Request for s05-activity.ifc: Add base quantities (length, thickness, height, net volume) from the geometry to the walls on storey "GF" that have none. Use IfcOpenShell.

First a look at what the model holds.

```python
import ifcopenshell
import ifcopenshell.util.element
import ifcopenshell.util.unit

model = ifcopenshell.open("s05-activity.ifc")
print(model.schema)
for unit_type in ("LENGTHUNIT", "AREAUNIT", "VOLUMEUNIT"):
    print(unit_type, ifcopenshell.util.unit.calculate_unit_scale(model, unit_type))
storey = next(s for s in model.by_type("IfcBuildingStorey") if s.Name == "GF")
walls = [e for e in ifcopenshell.util.element.get_decomposition(storey) if e.is_a("IfcWall")]
for e in sorted(walls, key=lambda e: e.id()):
    print(e.id(), e.is_a(), e.Name, list(ifcopenshell.util.element.get_psets(e, qtos_only=True)), sep=" | ")
```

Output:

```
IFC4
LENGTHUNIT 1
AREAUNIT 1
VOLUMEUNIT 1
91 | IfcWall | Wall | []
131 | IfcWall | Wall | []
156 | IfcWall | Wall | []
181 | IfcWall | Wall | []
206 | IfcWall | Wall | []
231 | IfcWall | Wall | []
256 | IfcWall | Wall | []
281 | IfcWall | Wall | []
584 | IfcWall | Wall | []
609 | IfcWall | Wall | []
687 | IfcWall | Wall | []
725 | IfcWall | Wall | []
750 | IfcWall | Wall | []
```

```python
import ifcopenshell
import ifcopenshell.api.pset
import ifcopenshell.geom
import ifcopenshell.util.element
import ifcopenshell.util.shape
import ifcopenshell.util.unit

model = ifcopenshell.open("s05-activity.ifc")
unit_scale = ifcopenshell.util.unit.calculate_unit_scale(model)
volume_scale = ifcopenshell.util.unit.calculate_unit_scale(model, "VOLUMEUNIT")
settings = ifcopenshell.geom.settings()

storey = next(s for s in model.by_type("IfcBuildingStorey") if s.Name == "GF")
walls = [e for e in ifcopenshell.util.element.get_decomposition(storey) if e.is_a("IfcWall")]

for e in sorted(walls, key=lambda e: e.id()):
    if ifcopenshell.util.element.get_psets(e, qtos_only=True, should_inherit=False):
        continue
    # Geometry comes back in metres, in the element's own axes.
    shape = ifcopenshell.geom.create_shape(settings, e)
    values = {
        "Length": ifcopenshell.util.shape.get_x(shape.geometry) / unit_scale,
        "Width": ifcopenshell.util.shape.get_y(shape.geometry) / unit_scale,
        "Height": ifcopenshell.util.shape.get_z(shape.geometry) / unit_scale,
        "NetVolume": ifcopenshell.util.shape.get_volume(shape.geometry) / volume_scale,
    }
    qto = ifcopenshell.api.pset.add_qto(model, product=e, name="Qto_WallBaseQuantities")
    ifcopenshell.api.pset.edit_qto(model, qto=qto, properties=values)
    print(e.id(), {k: round(v, 3) for k, v in values.items()})

model.write("s05-activity_updated.ifc")
```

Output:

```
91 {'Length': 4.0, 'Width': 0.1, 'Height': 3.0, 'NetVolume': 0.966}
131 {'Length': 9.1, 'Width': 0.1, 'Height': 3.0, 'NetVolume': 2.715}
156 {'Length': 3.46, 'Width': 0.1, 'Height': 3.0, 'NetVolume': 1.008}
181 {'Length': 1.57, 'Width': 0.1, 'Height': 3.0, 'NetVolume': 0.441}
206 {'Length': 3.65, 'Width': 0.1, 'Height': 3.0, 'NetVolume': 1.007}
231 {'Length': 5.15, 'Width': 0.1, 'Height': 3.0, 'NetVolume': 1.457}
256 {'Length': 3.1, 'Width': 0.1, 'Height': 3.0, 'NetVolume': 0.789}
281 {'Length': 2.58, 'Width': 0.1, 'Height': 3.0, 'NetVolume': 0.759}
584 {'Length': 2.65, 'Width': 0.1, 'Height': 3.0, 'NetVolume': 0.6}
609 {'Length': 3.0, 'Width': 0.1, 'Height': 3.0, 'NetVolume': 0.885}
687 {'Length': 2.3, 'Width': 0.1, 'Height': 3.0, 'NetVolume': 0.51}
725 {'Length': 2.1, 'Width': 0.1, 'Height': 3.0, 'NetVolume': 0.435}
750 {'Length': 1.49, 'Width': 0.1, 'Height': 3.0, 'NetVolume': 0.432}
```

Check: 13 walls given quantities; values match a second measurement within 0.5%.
